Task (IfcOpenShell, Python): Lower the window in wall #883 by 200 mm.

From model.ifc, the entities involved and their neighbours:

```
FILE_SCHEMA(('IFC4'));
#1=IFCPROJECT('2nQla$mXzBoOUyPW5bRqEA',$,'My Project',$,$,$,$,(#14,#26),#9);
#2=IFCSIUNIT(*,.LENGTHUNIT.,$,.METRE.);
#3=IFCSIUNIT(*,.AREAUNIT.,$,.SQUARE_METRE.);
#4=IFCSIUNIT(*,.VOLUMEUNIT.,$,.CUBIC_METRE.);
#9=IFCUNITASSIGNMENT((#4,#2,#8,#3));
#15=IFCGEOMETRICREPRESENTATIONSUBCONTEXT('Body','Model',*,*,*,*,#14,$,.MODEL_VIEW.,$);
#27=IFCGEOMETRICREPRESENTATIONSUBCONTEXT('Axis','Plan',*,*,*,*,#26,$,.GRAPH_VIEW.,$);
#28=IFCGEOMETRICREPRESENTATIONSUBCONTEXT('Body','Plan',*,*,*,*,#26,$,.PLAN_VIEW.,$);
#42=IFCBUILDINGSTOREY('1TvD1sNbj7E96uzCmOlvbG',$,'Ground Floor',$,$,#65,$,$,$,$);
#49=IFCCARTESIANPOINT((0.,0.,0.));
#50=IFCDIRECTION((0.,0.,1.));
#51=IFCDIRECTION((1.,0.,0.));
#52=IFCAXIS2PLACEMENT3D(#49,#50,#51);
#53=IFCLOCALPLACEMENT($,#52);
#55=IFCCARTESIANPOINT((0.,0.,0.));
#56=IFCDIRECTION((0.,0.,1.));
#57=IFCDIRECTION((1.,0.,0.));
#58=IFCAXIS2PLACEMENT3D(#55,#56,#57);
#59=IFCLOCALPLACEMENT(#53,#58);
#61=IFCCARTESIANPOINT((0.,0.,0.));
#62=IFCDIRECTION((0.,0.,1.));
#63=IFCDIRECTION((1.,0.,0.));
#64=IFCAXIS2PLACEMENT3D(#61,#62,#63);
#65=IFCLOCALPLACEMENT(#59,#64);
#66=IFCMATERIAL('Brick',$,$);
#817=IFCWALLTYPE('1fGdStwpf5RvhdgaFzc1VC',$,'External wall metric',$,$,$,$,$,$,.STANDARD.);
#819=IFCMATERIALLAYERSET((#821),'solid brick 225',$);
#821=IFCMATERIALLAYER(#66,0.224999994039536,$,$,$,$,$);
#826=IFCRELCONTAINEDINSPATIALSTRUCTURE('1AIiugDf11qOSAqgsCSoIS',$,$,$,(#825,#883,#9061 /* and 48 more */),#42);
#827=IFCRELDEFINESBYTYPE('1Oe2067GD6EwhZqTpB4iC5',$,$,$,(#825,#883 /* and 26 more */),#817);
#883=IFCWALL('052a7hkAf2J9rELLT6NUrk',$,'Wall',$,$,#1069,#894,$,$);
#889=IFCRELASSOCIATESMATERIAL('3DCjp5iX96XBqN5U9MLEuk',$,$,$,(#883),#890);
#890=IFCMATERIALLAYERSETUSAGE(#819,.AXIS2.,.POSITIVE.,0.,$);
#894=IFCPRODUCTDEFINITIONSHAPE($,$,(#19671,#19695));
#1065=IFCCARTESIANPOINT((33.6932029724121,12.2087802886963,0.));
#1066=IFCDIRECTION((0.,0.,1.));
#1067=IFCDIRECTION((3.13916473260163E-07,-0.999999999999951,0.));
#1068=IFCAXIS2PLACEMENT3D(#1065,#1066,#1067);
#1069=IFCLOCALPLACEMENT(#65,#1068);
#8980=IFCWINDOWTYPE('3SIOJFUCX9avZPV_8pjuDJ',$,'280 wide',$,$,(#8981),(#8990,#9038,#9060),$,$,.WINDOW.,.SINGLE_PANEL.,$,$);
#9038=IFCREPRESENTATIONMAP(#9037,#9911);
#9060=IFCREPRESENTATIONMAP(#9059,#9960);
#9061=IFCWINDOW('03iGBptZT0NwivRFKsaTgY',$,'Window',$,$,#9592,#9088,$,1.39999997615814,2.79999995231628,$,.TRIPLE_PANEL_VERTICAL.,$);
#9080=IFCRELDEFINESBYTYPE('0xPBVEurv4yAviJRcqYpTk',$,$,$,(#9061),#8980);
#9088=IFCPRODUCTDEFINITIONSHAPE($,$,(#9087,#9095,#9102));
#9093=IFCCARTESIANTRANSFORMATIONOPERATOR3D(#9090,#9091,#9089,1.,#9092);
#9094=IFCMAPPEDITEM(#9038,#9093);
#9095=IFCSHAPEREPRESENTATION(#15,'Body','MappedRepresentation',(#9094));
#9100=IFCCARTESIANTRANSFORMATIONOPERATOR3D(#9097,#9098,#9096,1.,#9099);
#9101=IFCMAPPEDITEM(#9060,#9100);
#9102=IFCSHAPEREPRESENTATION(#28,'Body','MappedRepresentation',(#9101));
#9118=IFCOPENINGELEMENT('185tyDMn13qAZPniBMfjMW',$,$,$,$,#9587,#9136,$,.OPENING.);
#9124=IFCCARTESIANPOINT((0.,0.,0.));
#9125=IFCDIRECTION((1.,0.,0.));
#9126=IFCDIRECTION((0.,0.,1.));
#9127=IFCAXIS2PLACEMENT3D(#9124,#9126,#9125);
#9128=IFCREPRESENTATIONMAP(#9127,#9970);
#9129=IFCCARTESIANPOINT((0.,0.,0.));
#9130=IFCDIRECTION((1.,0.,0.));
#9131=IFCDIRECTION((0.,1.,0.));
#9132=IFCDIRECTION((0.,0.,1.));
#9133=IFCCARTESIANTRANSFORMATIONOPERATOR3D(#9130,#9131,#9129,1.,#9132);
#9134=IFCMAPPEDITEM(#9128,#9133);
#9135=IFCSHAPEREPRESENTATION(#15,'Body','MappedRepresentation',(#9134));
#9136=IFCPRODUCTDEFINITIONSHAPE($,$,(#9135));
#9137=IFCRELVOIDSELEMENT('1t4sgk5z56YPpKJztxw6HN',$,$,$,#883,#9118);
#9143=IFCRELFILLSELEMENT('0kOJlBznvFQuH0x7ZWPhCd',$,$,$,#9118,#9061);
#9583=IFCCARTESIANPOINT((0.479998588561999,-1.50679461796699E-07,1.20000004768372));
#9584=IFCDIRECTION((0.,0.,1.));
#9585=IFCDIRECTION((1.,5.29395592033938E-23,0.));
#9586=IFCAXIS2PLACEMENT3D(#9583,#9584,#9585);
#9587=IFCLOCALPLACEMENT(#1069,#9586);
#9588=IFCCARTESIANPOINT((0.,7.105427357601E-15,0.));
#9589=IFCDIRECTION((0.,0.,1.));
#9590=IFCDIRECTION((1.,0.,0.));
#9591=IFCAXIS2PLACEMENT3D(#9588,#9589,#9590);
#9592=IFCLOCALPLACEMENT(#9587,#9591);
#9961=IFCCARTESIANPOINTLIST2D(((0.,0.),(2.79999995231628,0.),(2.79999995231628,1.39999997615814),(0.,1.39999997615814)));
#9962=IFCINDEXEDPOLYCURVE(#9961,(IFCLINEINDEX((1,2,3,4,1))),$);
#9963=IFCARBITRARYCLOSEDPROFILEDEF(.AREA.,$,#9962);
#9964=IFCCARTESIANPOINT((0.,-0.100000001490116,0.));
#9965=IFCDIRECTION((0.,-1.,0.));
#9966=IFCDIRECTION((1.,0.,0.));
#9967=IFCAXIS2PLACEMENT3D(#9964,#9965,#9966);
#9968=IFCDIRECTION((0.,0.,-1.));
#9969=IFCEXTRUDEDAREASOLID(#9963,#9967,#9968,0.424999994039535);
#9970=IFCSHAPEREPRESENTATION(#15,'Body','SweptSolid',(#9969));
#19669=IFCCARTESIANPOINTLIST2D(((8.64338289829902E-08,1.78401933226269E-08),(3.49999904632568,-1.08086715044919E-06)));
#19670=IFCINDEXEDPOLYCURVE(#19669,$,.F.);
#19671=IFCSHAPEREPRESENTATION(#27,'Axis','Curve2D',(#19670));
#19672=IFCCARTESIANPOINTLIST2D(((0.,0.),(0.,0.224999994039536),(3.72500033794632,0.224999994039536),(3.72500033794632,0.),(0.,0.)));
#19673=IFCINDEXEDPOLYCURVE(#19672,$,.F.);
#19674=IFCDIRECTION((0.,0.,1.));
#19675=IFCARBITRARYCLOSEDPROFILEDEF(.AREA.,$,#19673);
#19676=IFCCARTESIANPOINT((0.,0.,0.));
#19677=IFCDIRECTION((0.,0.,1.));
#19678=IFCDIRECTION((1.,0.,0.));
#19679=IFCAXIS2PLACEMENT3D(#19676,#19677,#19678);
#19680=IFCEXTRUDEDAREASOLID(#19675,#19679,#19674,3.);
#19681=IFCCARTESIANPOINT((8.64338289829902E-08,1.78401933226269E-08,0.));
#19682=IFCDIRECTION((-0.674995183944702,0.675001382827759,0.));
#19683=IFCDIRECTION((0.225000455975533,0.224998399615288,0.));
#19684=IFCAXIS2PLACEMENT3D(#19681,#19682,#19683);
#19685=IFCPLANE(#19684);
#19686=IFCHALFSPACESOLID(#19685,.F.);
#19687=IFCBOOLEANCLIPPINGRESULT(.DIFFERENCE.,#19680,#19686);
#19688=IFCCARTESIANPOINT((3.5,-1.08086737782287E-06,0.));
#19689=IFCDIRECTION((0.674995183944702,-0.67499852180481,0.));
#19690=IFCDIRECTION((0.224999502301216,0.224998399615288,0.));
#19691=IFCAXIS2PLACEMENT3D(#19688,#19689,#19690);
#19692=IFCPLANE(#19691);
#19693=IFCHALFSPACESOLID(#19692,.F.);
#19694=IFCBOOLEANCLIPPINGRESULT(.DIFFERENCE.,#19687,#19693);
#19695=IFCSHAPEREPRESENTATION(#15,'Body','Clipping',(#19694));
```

```python
import numpy as np
import ifcopenshell
import ifcopenshell.api.geometry
import ifcopenshell.util.placement
import ifcopenshell.util.unit

model = ifcopenshell.open("model.ifc")
unit_scale = ifcopenshell.util.unit.calculate_unit_scale(model)

window = model.by_guid("03iGBptZT0NwivRFKsaTgY")
opening = window.FillsVoids[0].RelatingOpeningElement
dz = -0.2

shift = np.array([0.0, 0.0, dz])
# The window is placed relative to its opening, so it follows when the opening moves.
matrix = ifcopenshell.util.placement.get_local_placement(opening.ObjectPlacement)
matrix[:3, 3] += shift
ifcopenshell.api.geometry.edit_object_placement(
    model, product=opening, matrix=matrix, is_si=False, should_transform_children=True
)

print(f"moved by {dz * unit_scale:+.3f} m")

model.write("model_edited.ifc")
```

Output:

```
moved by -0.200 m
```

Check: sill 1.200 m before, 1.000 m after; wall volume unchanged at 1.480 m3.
